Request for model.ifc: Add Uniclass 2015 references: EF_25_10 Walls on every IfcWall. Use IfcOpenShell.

First a look at what the model holds.

```python
import ifcopenshell

model = ifcopenshell.open("model.ifc")
print(model.schema)
print("classifications:", [c.Name for c in model.by_type("IfcClassification")])
for ifc_class in ("IfcDoor", "IfcRoof", "IfcStair", "IfcWall", "IfcWindow"):
    print(ifc_class, len(model.by_type(ifc_class)))
```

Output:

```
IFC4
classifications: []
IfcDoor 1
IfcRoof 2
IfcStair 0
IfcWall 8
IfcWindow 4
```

```python
import ifcopenshell
import ifcopenshell.api.classification

model = ifcopenshell.open("model.ifc")

system = ifcopenshell.api.classification.add_classification(model, classification="Uniclass 2015")

codes = {
    "IfcWall": ("EF_25_10", "Walls"),
}
for ifc_class, (code, name) in codes.items():
    products = model.by_type(ifc_class)
    ifcopenshell.api.classification.add_reference(
        model, products=products, classification=system, identification=code, name=name
    )
    print(code, len(products))

model.write("model-out.ifc")
```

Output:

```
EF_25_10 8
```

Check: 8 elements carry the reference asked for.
